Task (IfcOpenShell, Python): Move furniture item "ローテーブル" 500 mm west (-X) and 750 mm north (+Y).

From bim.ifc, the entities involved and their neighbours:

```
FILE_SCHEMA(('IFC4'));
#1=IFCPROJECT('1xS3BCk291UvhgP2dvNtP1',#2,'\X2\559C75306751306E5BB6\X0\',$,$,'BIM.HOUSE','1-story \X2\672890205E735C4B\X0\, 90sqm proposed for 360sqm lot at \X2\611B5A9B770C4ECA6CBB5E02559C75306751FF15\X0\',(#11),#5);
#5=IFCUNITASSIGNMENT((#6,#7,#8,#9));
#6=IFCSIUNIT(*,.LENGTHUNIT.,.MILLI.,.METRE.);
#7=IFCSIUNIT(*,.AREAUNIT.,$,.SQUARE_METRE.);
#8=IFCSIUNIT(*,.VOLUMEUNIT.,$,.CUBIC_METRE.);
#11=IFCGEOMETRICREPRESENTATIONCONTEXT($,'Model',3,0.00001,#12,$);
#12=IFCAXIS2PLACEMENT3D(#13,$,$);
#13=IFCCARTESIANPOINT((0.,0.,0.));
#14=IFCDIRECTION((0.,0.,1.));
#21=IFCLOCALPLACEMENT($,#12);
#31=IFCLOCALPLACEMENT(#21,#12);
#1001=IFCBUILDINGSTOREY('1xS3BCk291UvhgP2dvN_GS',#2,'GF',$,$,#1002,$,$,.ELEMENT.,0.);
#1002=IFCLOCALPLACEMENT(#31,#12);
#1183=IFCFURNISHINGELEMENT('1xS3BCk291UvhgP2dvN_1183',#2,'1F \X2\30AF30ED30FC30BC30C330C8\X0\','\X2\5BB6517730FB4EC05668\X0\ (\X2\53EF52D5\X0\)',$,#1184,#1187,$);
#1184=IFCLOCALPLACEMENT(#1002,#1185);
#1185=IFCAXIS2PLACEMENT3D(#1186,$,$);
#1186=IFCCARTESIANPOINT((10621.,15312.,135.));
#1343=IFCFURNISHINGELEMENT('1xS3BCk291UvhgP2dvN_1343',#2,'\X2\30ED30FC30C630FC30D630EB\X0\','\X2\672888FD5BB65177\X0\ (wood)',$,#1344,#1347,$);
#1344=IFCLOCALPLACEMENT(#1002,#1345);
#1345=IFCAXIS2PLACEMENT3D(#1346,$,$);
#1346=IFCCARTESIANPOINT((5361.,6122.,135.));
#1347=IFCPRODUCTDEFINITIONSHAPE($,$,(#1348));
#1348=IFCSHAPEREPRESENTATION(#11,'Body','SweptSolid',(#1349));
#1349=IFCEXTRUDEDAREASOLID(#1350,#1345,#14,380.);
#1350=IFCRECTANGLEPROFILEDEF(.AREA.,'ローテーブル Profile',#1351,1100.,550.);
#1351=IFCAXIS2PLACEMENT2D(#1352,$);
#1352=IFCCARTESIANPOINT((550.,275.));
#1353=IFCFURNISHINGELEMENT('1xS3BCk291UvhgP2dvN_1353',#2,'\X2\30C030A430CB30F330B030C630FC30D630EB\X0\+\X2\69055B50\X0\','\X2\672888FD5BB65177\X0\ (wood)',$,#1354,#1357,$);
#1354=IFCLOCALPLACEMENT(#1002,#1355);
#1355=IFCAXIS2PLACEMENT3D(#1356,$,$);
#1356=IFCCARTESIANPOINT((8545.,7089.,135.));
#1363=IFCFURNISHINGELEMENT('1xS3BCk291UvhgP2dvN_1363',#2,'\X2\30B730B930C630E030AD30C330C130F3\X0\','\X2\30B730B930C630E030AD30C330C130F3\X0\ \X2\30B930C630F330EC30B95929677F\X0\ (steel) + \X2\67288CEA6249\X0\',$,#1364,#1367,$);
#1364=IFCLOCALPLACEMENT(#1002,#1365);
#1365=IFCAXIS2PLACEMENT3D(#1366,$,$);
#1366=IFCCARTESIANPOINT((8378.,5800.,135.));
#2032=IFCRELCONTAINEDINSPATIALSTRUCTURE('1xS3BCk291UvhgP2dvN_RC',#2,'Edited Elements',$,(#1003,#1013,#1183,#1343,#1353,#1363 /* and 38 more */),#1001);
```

```python
import ifcopenshell
import ifcopenshell.api.geometry
import ifcopenshell.util.placement
import ifcopenshell.util.unit

model = ifcopenshell.open("bim.ifc")
unit_scale = ifcopenshell.util.unit.calculate_unit_scale(model)

item = model.by_guid("1xS3BCk291UvhgP2dvN_1343")
matrix = ifcopenshell.util.placement.get_local_placement(item.ObjectPlacement)
matrix[0, 3] -= 0.5 / unit_scale
matrix[1, 3] += 0.75 / unit_scale
ifcopenshell.api.geometry.edit_object_placement(model, product=item, matrix=matrix, is_si=False)

print(ifcopenshell.util.placement.get_local_placement(item.ObjectPlacement).round(3) + 0.0)

model.write("bim_v2.ifc")
```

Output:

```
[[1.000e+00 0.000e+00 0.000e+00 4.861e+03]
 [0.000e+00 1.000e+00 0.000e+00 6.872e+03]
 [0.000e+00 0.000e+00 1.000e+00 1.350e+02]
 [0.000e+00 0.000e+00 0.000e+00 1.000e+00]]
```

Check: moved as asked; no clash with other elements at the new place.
